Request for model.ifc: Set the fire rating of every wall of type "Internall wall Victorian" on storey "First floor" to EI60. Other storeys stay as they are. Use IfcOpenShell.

First a look at what the model holds.

```python
import ifcopenshell
import ifcopenshell.util.element

model = ifcopenshell.open("model.ifc")
print(model.schema)
storey = next(s for s in model.by_type("IfcBuildingStorey") if s.Name == "First floor")
walls = [e for e in ifcopenshell.util.element.get_decomposition(storey) if e.is_a("IfcWall")]
seen = {}
for e in walls:
    element_type = ifcopenshell.util.element.get_type(e)
    key = (element_type.Name if element_type != e and element_type else None, ifcopenshell.util.element.get_pset(e, "Pset_WallCommon", "FireRating"))
    seen[key] = seen.get(key, 0) + 1
for (name, value), count in sorted(seen.items(), key=str):
    print(count, "x", name, "|", value)
```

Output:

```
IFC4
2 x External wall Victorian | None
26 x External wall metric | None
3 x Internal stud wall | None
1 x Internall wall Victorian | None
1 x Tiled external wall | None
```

```python
import ifcopenshell
import ifcopenshell.api.pset
import ifcopenshell.util.element

model = ifcopenshell.open("model.ifc")

storey = next(s for s in model.by_type("IfcBuildingStorey") if s.Name == "First floor")
walls = [e for e in ifcopenshell.util.element.get_decomposition(storey) if e.is_a("IfcWall")]

count = 0
for e in walls:
    element_type = ifcopenshell.util.element.get_type(e)
    if element_type in (None, e) or element_type.Name != "Internall wall Victorian":
        continue
    # add_pset returns the element's existing set when there is one.
    pset = ifcopenshell.api.pset.add_pset(model, product=e, name="Pset_WallCommon")
    ifcopenshell.api.pset.edit_pset(model, pset=pset, properties={"FireRating": "EI60"})
    count += 1

print(count, "walls updated")

model.write("model_updated.ifc")
```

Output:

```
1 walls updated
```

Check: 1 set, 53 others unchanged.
